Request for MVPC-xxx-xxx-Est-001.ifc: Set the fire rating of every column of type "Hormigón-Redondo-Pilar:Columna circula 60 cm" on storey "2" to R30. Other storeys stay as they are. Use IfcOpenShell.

First a look at what the model holds.

```python
import ifcopenshell
import ifcopenshell.util.element

model = ifcopenshell.open("MVPC-xxx-xxx-Est-001.ifc")
print(model.schema)
storey = next(s for s in model.by_type("IfcBuildingStorey") if s.Name == "2")
columns = [e for e in ifcopenshell.util.element.get_decomposition(storey) if e.is_a("IfcColumn")]
seen = {}
for e in columns:
    element_type = ifcopenshell.util.element.get_type(e)
    key = (element_type.Name if element_type != e and element_type else None, ifcopenshell.util.element.get_pset(e, "Pset_ColumnCommon", "FireRating"))
    seen[key] = seen.get(key, 0) + 1
for (name, value), count in sorted(seen.items(), key=str):
    print(count, "x", name, "|", value)
```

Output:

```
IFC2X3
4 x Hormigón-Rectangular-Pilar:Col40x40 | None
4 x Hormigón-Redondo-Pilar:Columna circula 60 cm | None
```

```python
import ifcopenshell
import ifcopenshell.api.pset
import ifcopenshell.util.element

model = ifcopenshell.open("MVPC-xxx-xxx-Est-001.ifc")

storey = next(s for s in model.by_type("IfcBuildingStorey") if s.Name == "2")
columns = [e for e in ifcopenshell.util.element.get_decomposition(storey) if e.is_a("IfcColumn")]

count = 0
for e in columns:
    element_type = ifcopenshell.util.element.get_type(e)
    if element_type in (None, e) or element_type.Name != "Hormigón-Redondo-Pilar:Columna circula 60 cm":
        continue
    # add_pset returns the element's existing set when there is one.
    pset = ifcopenshell.api.pset.add_pset(model, product=e, name="Pset_ColumnCommon")
    ifcopenshell.api.pset.edit_pset(model, pset=pset, properties={"FireRating": "R30"})
    count += 1

print(count, "columns updated")

model.write("MVPC-xxx-xxx-Est-001_edited.ifc")
```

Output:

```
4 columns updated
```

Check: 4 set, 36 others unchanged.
